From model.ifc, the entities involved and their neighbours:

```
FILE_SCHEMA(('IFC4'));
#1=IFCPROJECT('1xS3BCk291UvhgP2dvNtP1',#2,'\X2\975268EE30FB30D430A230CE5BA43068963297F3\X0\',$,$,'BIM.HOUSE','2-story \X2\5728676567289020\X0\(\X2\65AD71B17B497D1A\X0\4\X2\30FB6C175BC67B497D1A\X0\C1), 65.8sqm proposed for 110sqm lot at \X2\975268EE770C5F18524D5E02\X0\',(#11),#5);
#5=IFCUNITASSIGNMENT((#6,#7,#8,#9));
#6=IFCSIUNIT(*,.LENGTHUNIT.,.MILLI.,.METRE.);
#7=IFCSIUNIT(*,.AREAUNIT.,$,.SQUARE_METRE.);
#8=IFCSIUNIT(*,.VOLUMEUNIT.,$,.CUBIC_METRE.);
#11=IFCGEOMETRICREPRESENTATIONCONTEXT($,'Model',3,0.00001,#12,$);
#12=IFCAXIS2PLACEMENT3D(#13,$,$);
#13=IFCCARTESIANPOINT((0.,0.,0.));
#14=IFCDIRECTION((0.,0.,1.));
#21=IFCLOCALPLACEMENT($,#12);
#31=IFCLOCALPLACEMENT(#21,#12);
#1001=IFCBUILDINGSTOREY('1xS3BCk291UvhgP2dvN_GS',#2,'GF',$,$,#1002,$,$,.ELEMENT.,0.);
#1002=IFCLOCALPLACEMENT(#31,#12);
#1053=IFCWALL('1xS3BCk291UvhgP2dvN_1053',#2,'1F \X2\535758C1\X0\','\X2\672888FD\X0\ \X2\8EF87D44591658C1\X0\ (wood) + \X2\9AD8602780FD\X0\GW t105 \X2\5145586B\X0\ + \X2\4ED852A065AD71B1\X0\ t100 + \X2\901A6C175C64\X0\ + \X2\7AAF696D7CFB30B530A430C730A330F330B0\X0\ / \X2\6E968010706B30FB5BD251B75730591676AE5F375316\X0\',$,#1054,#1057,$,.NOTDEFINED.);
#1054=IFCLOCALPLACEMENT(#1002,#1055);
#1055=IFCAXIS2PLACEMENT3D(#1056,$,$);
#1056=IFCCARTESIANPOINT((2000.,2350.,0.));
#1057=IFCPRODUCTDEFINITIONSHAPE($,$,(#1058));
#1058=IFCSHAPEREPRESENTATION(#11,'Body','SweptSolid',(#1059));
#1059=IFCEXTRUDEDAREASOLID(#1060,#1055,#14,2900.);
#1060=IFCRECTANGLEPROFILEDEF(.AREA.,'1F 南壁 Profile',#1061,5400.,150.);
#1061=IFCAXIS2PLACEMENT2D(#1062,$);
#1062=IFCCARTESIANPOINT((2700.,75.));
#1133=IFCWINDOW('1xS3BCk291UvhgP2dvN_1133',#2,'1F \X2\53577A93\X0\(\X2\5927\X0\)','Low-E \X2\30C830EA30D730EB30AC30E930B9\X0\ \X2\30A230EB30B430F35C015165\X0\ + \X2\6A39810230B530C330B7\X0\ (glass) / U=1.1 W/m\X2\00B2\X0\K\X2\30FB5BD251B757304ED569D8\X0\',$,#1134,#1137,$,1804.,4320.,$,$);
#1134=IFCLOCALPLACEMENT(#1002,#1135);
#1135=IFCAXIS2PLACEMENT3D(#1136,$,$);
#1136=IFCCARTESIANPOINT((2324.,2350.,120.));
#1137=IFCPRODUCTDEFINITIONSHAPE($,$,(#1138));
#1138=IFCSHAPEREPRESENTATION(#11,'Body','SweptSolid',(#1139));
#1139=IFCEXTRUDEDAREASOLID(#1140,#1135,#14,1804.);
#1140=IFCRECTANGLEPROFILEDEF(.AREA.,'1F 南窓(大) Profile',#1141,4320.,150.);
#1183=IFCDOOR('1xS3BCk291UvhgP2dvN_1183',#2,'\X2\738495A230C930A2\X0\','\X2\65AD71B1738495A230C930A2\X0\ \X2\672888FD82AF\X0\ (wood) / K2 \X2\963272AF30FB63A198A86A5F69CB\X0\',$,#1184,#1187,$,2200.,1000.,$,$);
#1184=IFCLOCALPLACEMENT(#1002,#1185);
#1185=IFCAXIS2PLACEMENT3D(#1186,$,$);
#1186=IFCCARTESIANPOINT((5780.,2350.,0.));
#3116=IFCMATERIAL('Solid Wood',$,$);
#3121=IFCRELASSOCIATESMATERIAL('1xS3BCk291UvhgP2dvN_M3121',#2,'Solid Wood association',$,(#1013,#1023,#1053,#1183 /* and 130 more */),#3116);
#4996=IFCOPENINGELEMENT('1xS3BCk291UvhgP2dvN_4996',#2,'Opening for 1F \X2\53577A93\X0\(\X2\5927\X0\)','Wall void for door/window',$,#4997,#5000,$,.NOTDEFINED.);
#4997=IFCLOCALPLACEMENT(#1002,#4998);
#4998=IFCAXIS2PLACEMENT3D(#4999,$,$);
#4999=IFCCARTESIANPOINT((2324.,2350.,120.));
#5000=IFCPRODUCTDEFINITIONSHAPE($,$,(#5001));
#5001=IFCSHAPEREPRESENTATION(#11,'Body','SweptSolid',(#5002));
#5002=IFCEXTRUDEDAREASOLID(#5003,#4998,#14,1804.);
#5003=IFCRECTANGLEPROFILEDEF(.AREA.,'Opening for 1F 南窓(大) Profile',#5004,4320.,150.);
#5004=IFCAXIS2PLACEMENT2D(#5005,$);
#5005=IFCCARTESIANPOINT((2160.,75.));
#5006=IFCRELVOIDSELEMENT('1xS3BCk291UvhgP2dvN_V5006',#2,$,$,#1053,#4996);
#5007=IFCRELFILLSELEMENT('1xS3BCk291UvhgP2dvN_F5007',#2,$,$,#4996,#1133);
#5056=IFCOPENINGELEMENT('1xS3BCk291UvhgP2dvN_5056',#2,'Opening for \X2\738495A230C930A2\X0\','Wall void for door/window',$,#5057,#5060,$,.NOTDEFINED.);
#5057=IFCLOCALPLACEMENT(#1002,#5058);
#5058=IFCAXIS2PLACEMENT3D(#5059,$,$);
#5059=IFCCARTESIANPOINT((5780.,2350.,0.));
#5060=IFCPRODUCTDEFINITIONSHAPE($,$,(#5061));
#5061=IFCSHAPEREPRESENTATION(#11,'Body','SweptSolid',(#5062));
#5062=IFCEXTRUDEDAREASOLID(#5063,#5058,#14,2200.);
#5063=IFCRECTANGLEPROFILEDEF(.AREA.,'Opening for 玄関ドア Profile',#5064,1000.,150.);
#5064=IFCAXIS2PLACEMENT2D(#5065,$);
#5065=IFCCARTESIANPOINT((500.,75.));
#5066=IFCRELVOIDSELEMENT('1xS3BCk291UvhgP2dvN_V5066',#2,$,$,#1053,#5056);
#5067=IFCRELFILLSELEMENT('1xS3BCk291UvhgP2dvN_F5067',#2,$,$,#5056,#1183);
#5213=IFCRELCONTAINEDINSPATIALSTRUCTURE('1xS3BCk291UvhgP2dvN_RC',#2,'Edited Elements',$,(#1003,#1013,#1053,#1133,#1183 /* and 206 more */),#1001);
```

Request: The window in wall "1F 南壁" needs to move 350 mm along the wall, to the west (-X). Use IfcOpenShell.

```python
import ifcopenshell
import ifcopenshell.api.geometry
import ifcopenshell.util.placement
import ifcopenshell.util.unit

model = ifcopenshell.open("model.ifc")
unit_scale = ifcopenshell.util.unit.calculate_unit_scale(model)

window = model.by_guid("1xS3BCk291UvhgP2dvN_1133")
opening = window.FillsVoids[0].RelatingOpeningElement
wall = opening.VoidsElements[0].RelatingBuildingElement

wall_matrix = ifcopenshell.util.placement.get_local_placement(wall.ObjectPlacement)
shift = wall_matrix[:3, 0] * -0.35 / unit_scale
before = ifcopenshell.util.placement.get_local_placement(window.ObjectPlacement)[:3, 3].copy()

# The window is not placed relative to its opening, so move both.
for product in (opening, window):
    matrix = ifcopenshell.util.placement.get_local_placement(product.ObjectPlacement)
    matrix[:3, 3] += shift
    ifcopenshell.api.geometry.edit_object_placement(model, product=product, matrix=matrix, is_si=False)

after = ifcopenshell.util.placement.get_local_placement(window.ObjectPlacement)[:3, 3]
print("window moved by", (after - before).round(3) + 0.0)

model.write("model-out.ifc")
```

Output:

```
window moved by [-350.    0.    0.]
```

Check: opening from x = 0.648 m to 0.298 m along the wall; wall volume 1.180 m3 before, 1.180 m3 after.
